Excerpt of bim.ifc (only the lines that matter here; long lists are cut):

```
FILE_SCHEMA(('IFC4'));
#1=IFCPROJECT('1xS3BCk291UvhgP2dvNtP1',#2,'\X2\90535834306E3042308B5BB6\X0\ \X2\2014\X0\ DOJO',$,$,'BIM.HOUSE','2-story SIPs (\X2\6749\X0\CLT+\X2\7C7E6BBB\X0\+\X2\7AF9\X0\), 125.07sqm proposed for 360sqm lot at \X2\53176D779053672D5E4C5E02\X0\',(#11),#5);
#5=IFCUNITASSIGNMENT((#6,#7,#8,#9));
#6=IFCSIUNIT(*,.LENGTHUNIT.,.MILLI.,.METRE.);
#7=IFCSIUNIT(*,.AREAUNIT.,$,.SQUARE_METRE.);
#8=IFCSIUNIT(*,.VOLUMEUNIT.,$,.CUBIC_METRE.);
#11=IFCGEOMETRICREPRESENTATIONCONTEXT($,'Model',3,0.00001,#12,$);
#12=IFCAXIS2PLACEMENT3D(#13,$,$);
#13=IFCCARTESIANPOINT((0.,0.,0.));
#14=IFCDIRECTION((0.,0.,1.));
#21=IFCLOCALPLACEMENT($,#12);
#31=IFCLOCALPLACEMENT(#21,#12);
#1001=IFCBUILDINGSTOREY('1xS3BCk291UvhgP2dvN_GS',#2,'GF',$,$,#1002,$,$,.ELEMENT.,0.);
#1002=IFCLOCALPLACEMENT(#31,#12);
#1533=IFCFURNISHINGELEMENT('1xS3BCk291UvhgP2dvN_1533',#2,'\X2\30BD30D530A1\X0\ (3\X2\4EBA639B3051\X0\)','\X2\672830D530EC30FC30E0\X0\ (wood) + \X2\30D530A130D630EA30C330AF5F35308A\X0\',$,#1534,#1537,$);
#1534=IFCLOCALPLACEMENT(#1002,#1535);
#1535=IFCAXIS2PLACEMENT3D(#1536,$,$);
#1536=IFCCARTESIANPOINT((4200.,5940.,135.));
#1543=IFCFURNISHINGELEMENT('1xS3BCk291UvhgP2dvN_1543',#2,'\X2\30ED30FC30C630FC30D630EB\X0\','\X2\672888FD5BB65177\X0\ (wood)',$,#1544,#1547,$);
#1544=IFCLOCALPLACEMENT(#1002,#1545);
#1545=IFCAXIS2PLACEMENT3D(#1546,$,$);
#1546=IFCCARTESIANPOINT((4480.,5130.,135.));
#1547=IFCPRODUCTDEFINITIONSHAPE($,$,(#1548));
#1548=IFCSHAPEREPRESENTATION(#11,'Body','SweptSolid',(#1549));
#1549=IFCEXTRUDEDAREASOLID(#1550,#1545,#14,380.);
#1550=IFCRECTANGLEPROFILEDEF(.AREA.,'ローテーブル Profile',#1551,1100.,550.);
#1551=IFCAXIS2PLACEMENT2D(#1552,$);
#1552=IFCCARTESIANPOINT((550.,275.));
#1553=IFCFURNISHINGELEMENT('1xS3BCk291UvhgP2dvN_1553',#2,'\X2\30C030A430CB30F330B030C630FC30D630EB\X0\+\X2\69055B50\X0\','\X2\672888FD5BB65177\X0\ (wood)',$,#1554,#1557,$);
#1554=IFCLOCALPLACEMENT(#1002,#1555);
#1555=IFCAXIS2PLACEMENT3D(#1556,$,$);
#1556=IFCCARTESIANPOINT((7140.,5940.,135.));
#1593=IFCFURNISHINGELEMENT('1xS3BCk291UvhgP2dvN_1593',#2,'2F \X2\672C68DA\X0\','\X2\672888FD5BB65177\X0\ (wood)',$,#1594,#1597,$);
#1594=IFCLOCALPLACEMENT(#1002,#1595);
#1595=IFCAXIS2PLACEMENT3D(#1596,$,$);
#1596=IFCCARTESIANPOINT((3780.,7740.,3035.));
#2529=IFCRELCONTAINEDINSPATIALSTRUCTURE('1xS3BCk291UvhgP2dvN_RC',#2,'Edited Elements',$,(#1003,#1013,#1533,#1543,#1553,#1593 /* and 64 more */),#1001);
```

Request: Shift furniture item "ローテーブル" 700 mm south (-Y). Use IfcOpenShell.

```python
import ifcopenshell
import ifcopenshell.api.geometry
import ifcopenshell.util.placement
import ifcopenshell.util.unit

model = ifcopenshell.open("bim.ifc")
unit_scale = ifcopenshell.util.unit.calculate_unit_scale(model)

item = model.by_guid("1xS3BCk291UvhgP2dvN_1543")
matrix = ifcopenshell.util.placement.get_local_placement(item.ObjectPlacement)
matrix[1, 3] -= 0.7 / unit_scale
ifcopenshell.api.geometry.edit_object_placement(model, product=item, matrix=matrix, is_si=False)

print(ifcopenshell.util.placement.get_local_placement(item.ObjectPlacement).round(3) + 0.0)

model.write("bim_v2.ifc")
```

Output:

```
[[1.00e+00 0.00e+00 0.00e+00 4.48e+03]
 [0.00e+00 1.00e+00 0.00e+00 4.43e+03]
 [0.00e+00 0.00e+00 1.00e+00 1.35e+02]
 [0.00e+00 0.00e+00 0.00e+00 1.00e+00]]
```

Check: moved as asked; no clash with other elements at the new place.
